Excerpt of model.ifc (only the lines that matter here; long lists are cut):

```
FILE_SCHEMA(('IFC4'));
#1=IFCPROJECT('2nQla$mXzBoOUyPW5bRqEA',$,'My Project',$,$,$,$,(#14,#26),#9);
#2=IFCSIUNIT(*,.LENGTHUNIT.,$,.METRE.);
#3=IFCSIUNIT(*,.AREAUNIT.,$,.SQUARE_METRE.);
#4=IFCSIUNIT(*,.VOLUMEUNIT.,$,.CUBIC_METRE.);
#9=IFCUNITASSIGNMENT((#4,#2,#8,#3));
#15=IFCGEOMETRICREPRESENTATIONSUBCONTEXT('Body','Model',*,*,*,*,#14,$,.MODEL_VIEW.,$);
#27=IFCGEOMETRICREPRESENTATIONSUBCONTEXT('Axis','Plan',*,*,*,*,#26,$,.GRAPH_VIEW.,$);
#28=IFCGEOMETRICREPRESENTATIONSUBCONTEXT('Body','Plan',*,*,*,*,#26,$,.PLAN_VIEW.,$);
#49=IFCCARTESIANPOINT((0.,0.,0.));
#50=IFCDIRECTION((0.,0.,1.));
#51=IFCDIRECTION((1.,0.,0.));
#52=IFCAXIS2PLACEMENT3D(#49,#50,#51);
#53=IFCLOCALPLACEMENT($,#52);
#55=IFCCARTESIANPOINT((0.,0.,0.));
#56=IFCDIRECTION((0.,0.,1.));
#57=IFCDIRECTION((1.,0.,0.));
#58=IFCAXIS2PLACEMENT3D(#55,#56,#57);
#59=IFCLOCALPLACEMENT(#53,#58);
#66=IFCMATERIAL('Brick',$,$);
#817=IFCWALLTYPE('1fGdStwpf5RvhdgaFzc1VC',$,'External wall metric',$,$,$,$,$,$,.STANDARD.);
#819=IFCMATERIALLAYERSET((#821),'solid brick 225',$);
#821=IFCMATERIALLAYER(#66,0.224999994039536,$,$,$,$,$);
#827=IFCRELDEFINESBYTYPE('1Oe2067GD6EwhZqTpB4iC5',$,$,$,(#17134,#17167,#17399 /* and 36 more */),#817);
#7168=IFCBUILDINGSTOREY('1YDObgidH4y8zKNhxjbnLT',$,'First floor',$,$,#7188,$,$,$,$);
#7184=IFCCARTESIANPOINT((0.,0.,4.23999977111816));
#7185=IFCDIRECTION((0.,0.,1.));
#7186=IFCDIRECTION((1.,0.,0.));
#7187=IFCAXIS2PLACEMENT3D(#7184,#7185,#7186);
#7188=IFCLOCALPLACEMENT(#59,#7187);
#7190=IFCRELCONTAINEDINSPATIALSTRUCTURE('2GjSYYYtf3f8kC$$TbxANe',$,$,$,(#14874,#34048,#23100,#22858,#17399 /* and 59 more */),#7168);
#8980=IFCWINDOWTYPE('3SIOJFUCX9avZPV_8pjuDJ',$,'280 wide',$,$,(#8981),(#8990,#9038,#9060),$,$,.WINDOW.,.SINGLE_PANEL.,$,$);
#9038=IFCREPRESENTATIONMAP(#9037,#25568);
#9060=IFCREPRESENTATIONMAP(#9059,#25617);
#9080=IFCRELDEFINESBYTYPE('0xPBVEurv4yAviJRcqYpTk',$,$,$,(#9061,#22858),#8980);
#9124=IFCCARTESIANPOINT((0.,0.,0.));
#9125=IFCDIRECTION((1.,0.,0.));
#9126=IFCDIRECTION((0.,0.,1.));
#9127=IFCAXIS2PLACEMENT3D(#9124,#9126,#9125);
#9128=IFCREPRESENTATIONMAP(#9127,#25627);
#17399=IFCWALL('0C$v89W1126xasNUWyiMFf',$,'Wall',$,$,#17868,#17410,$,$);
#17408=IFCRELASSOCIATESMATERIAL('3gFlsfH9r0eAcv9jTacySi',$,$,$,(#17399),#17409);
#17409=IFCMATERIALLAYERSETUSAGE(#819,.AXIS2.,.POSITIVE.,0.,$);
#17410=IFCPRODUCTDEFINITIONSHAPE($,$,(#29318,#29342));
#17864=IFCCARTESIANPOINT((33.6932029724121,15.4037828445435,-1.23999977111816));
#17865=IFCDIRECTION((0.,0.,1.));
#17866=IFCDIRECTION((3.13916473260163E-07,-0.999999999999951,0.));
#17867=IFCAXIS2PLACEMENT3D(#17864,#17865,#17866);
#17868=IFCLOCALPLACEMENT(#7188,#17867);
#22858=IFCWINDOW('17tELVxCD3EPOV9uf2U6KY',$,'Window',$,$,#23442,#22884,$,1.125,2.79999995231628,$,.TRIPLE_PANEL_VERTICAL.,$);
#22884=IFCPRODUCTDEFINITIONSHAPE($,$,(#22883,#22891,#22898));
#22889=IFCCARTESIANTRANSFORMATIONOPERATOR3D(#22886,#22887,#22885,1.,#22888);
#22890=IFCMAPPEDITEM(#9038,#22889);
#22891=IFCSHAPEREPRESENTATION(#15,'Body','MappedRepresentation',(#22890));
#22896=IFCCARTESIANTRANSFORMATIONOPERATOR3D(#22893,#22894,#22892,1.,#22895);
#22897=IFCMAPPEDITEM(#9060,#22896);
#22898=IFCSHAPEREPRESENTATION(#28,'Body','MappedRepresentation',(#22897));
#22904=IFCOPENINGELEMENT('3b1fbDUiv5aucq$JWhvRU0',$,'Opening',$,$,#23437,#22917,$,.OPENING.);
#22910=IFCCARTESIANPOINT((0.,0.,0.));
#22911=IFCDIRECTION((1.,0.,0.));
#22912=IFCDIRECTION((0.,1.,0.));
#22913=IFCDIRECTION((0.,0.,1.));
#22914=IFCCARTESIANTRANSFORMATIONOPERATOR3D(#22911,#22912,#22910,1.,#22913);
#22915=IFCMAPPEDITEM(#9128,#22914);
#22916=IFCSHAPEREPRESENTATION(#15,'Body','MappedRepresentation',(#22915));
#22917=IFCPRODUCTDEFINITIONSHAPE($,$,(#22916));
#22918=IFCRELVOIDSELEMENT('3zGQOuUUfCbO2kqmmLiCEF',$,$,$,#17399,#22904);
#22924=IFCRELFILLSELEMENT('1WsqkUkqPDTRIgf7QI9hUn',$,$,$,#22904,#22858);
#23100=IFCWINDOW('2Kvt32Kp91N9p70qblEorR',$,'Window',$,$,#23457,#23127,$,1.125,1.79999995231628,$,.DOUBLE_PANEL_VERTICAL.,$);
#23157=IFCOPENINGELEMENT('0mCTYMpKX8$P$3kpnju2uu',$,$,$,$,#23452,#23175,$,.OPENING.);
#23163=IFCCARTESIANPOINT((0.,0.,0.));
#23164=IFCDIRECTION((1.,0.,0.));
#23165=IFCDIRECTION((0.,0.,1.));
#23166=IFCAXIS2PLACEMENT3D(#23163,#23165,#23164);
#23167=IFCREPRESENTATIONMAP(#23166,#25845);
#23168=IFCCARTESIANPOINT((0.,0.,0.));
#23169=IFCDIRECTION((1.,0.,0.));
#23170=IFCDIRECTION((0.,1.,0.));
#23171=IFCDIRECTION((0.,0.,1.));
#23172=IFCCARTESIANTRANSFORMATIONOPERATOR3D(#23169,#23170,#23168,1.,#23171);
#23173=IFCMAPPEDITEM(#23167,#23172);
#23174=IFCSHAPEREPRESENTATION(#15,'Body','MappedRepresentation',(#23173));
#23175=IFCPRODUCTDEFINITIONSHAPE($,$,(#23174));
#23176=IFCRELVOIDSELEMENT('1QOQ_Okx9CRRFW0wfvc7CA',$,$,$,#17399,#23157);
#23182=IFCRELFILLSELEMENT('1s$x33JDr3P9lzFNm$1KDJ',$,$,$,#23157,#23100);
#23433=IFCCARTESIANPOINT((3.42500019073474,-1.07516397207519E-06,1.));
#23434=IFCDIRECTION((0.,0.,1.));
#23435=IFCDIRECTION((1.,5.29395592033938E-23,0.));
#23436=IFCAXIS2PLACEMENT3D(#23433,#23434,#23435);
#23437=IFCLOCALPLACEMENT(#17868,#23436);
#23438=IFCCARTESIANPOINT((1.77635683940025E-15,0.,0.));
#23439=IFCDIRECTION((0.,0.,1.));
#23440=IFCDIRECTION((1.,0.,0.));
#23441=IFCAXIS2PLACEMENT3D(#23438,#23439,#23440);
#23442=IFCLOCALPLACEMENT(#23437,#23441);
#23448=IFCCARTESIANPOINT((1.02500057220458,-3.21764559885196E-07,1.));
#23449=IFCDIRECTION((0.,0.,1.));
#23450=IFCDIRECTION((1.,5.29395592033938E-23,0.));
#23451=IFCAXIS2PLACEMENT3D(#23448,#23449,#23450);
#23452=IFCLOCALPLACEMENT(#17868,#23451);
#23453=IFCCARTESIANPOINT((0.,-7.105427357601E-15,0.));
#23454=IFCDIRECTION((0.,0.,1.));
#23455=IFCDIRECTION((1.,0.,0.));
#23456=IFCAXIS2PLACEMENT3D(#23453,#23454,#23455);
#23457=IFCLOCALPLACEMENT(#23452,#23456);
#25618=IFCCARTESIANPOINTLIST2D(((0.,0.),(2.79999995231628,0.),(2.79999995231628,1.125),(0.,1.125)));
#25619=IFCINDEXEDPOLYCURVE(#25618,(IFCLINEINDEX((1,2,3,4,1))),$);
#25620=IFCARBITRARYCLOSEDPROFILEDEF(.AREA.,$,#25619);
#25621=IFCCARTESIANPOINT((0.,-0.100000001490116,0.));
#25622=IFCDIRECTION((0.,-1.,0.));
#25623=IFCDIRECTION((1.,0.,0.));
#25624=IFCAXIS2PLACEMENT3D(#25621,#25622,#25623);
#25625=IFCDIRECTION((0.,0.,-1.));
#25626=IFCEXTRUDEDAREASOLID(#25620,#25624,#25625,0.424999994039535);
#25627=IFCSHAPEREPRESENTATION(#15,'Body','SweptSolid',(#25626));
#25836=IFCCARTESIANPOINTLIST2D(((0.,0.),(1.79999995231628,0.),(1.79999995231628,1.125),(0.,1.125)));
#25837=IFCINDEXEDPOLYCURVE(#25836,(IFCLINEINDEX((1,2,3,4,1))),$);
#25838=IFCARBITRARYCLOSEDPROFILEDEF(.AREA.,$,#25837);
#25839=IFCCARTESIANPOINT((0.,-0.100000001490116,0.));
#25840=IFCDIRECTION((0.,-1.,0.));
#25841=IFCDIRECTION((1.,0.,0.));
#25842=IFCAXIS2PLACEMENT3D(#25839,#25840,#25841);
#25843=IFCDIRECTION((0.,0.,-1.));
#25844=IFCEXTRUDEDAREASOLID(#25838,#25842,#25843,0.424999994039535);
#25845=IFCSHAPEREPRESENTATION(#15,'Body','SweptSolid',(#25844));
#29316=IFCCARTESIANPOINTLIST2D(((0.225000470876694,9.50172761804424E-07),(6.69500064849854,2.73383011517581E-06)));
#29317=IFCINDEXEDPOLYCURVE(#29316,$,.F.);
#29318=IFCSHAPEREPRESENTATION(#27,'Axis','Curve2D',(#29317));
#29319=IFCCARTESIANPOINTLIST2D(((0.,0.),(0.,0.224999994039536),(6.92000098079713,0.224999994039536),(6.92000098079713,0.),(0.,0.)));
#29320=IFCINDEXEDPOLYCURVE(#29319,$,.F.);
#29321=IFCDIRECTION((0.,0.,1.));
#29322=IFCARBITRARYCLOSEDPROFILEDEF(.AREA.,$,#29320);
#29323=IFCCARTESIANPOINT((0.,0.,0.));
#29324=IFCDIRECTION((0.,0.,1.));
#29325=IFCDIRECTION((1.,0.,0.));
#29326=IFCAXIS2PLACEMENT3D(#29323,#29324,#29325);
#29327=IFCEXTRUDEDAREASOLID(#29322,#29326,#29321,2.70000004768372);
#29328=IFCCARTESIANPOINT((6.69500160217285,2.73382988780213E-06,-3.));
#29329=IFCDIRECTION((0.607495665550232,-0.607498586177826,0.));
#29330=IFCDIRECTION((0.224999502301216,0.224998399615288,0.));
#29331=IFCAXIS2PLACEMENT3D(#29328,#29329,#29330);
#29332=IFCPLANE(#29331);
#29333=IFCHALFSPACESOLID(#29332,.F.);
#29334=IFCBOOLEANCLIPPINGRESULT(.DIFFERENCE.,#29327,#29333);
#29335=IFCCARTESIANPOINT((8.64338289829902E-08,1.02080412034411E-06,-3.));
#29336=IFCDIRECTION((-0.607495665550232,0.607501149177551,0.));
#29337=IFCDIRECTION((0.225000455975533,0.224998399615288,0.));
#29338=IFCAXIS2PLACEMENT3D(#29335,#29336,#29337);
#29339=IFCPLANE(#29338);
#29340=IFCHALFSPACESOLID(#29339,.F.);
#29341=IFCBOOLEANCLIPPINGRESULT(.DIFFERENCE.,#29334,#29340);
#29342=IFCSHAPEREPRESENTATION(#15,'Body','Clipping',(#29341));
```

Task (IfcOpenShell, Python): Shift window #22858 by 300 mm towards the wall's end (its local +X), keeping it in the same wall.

```python
import ifcopenshell
import ifcopenshell.api.geometry
import ifcopenshell.util.placement
import ifcopenshell.util.unit

model = ifcopenshell.open("model.ifc")
unit_scale = ifcopenshell.util.unit.calculate_unit_scale(model)

window = model.by_guid("17tELVxCD3EPOV9uf2U6KY")
opening = window.FillsVoids[0].RelatingOpeningElement
wall = opening.VoidsElements[0].RelatingBuildingElement

wall_matrix = ifcopenshell.util.placement.get_local_placement(wall.ObjectPlacement)
shift = wall_matrix[:3, 0] * 0.3 / unit_scale
before = ifcopenshell.util.placement.get_local_placement(window.ObjectPlacement)[:3, 3].copy()

# The window is placed relative to its opening, so it follows when the opening moves.
matrix = ifcopenshell.util.placement.get_local_placement(opening.ObjectPlacement)
matrix[:3, 3] += shift
ifcopenshell.api.geometry.edit_object_placement(
    model, product=opening, matrix=matrix, is_si=False, should_transform_children=True
)

after = ifcopenshell.util.placement.get_local_placement(window.ObjectPlacement)[:3, 3]
print("window moved by", (after - before).round(3) + 0.0)

model.write("model_edited.ifc")
```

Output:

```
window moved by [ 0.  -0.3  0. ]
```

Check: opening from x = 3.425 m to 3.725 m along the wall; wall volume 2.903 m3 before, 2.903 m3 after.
